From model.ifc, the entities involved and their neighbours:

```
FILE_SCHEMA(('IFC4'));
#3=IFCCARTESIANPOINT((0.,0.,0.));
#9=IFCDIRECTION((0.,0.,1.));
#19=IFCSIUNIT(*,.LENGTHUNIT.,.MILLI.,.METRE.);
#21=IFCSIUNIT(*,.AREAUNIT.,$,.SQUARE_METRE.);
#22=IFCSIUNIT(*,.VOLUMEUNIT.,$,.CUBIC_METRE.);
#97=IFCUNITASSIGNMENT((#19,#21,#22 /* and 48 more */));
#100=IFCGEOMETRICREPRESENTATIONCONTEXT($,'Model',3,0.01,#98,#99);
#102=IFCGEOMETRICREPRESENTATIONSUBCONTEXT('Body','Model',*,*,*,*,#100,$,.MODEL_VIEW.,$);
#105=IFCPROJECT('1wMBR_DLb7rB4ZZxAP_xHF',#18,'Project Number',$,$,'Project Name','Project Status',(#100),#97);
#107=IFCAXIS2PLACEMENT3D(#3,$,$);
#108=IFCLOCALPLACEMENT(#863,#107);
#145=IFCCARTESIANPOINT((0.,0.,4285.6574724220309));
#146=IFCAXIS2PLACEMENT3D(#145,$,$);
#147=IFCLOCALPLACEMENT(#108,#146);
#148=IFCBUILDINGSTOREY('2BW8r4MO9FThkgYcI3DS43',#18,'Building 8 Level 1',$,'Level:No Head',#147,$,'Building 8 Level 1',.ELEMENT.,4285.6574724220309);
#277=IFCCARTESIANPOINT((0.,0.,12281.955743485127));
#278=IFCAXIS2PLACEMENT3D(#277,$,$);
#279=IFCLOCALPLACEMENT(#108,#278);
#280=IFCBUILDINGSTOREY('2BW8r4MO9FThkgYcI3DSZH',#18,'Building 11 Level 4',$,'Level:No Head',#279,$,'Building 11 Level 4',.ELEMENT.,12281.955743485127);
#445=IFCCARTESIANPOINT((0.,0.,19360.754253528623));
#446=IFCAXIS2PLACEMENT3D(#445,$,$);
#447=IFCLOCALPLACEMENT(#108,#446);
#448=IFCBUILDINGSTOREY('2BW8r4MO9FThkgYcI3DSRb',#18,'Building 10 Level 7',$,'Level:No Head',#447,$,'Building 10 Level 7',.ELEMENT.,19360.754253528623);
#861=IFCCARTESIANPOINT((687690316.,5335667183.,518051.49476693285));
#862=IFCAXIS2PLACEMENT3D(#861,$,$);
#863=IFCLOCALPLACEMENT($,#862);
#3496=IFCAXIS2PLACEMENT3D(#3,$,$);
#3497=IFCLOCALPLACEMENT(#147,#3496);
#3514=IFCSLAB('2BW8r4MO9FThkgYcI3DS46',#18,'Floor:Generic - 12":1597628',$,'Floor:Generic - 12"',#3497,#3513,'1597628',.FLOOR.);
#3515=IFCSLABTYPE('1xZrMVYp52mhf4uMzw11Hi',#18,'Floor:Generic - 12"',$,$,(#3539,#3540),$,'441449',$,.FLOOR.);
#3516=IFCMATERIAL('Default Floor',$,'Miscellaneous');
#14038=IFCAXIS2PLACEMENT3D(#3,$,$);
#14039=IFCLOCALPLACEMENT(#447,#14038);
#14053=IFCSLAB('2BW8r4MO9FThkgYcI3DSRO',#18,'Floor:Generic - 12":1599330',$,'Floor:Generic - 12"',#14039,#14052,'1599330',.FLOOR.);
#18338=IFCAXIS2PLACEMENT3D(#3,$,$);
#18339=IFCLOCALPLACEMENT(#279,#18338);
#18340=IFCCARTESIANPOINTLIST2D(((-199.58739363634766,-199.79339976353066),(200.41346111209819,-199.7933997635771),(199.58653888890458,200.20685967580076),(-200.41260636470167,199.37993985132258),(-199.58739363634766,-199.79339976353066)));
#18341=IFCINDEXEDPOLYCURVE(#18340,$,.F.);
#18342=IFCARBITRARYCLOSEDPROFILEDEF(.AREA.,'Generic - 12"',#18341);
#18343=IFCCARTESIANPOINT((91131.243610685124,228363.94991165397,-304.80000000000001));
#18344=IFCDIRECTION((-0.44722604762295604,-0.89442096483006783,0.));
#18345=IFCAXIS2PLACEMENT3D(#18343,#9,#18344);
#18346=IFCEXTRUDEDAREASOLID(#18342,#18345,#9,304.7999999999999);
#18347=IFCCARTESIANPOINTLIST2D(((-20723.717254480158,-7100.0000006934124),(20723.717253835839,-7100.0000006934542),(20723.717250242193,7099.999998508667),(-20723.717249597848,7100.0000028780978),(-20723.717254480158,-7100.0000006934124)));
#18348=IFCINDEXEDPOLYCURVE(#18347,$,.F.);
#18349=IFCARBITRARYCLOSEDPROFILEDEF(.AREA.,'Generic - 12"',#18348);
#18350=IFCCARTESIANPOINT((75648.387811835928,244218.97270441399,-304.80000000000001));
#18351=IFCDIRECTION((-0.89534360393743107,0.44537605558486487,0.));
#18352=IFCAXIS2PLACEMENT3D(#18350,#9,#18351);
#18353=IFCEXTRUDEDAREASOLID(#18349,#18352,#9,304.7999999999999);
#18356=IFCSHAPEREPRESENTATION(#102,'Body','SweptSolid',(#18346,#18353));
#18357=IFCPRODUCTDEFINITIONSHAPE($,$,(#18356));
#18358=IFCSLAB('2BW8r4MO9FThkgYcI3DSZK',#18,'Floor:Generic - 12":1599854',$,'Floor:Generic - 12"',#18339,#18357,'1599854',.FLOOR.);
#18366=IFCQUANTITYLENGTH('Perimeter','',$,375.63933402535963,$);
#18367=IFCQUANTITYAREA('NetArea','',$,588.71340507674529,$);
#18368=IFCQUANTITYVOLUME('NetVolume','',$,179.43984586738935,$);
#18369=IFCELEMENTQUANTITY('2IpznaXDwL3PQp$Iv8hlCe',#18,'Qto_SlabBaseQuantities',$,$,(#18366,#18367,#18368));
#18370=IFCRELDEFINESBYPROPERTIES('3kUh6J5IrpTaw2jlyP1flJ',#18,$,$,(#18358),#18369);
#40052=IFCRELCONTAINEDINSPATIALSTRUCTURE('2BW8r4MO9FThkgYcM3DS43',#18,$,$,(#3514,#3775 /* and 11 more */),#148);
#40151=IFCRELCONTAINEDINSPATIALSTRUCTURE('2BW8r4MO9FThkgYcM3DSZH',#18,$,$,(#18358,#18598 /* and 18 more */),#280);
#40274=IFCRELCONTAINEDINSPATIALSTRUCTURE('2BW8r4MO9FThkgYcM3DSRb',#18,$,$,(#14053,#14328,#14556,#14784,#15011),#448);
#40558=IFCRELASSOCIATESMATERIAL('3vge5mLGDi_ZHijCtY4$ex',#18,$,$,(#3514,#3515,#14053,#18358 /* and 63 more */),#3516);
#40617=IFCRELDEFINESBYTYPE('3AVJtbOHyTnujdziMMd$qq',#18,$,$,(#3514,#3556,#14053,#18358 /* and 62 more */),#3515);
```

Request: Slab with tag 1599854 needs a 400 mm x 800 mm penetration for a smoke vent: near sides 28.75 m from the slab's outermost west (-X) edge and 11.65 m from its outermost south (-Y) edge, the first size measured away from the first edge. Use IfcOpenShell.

```python
import numpy as np
import ifcopenshell
import ifcopenshell.api.feature
import ifcopenshell.api.geometry
import ifcopenshell.api.pset
import ifcopenshell.api.root
import ifcopenshell.geom
import ifcopenshell.util.element
import ifcopenshell.util.placement
import ifcopenshell.util.representation
import ifcopenshell.util.shape
import ifcopenshell.util.unit

model = ifcopenshell.open("model.ifc")
unit_scale = ifcopenshell.util.unit.calculate_unit_scale(model)
area_scale = ifcopenshell.util.unit.calculate_unit_scale(model, "AREAUNIT")
volume_scale = ifcopenshell.util.unit.calculate_unit_scale(model, "VOLUMEUNIT")
settings = ifcopenshell.geom.settings()


def volume(element):
    """Net volume in cubic metres, openings subtracted."""
    shape = ifcopenshell.geom.create_shape(settings, element)
    return ifcopenshell.util.shape.get_volume(shape.geometry)


slab = model.by_guid("2BW8r4MO9FThkgYcI3DSZK")
before = volume(slab)

# Extent in the slab's own axes, in metres. The edges named are its -X and -Y sides.
slab_shape = ifcopenshell.geom.create_shape(settings, slab)
vertices = ifcopenshell.util.shape.get_vertices(slab_shape.geometry)
x_min, y_min, bottom = vertices.min(axis=0)
top = vertices[:, 2].max()

opening = ifcopenshell.api.root.create_entity(model, ifc_class="IfcOpeningElement", name="Smoke vent opening", predefined_type="OPENING")
context = ifcopenshell.util.representation.get_context(model, "Model", "Body", "MODEL_VIEW")
width, depth = 0.4, 0.8
outline = [(0.0, 0.0), (width, 0.0), (width, depth), (0.0, depth), (0.0, 0.0)]
# Overshoot both faces by 50 mm so the cut is clean.
shape = ifcopenshell.api.geometry.add_slab_representation(
    model, context=context, depth=top - bottom + 0.1, polyline=outline
)
ifcopenshell.api.geometry.assign_representation(model, product=opening, representation=shape)

matrix = ifcopenshell.util.placement.get_local_placement(slab.ObjectPlacement)
matrix[:, 3] = matrix @ np.append(np.array([x_min + 28.75, y_min + 11.65, bottom - 0.05]) / unit_scale, 1.0)
ifcopenshell.api.geometry.edit_object_placement(model, product=opening, matrix=matrix, is_si=False)
ifcopenshell.api.feature.add_feature(model, feature=opening, element=slab)

after = volume(slab)

# Update the slab's stored quantities.
qto = model.by_id(ifcopenshell.util.element.get_pset(slab, "Qto_SlabBaseQuantities", should_inherit=False)["id"])
ifcopenshell.api.pset.edit_qto(model, qto=qto, properties={
    "NetArea": after / (top - bottom) / area_scale,
    "NetVolume": after / volume_scale,
})

print(f"slab volume {before:.3f} -> {after:.3f} m3")

model.write("model_rev.ifc")
```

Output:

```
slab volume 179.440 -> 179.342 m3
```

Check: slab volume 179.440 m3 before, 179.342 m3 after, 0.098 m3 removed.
